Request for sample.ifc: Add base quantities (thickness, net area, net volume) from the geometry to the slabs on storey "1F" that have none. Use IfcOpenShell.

First a look at what the model holds.

```python
import ifcopenshell
import ifcopenshell.util.element
import ifcopenshell.util.unit

model = ifcopenshell.open("sample.ifc")
print(model.schema)
for unit_type in ("LENGTHUNIT", "AREAUNIT", "VOLUMEUNIT"):
    print(unit_type, ifcopenshell.util.unit.calculate_unit_scale(model, unit_type))
storey = next(s for s in model.by_type("IfcBuildingStorey") if s.Name == "1F")
slabs = [e for e in ifcopenshell.util.element.get_decomposition(storey) if e.is_a("IfcSlab")]
for e in sorted(slabs, key=lambda e: e.id()):
    print(e.id(), e.is_a(), e.Name, list(ifcopenshell.util.element.get_psets(e, qtos_only=True)), sep=" | ")
```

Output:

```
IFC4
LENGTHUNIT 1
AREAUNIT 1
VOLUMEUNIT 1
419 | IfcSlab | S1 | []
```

```python
import ifcopenshell
import ifcopenshell.api.pset
import ifcopenshell.geom
import ifcopenshell.util.element
import ifcopenshell.util.shape
import ifcopenshell.util.unit

model = ifcopenshell.open("sample.ifc")
unit_scale = ifcopenshell.util.unit.calculate_unit_scale(model)
area_scale = ifcopenshell.util.unit.calculate_unit_scale(model, "AREAUNIT")
volume_scale = ifcopenshell.util.unit.calculate_unit_scale(model, "VOLUMEUNIT")
settings = ifcopenshell.geom.settings()

storey = next(s for s in model.by_type("IfcBuildingStorey") if s.Name == "1F")
slabs = [e for e in ifcopenshell.util.element.get_decomposition(storey) if e.is_a("IfcSlab")]

for e in sorted(slabs, key=lambda e: e.id()):
    if ifcopenshell.util.element.get_psets(e, qtos_only=True, should_inherit=False):
        continue
    # Geometry comes back in metres, in the element's own axes.
    shape = ifcopenshell.geom.create_shape(settings, e)
    values = {
        "Width": ifcopenshell.util.shape.get_z(shape.geometry) / unit_scale,
        "NetArea": ifcopenshell.util.shape.get_footprint_area(shape.geometry) / area_scale,
        "NetVolume": ifcopenshell.util.shape.get_volume(shape.geometry) / volume_scale,
    }
    qto = ifcopenshell.api.pset.add_qto(model, product=e, name="Qto_SlabBaseQuantities")
    ifcopenshell.api.pset.edit_qto(model, qto=qto, properties=values)
    print(e.id(), {k: round(v, 3) for k, v in values.items()})

model.write("sample_edited.ifc")
```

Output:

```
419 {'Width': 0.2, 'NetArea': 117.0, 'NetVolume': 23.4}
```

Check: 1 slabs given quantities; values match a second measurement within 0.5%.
